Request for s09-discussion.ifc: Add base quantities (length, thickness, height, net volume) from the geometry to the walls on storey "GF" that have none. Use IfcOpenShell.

First a look at what the model holds.

```python
import ifcopenshell
import ifcopenshell.util.element
import ifcopenshell.util.unit

model = ifcopenshell.open("s09-discussion.ifc")
print(model.schema)
for unit_type in ("LENGTHUNIT", "AREAUNIT", "VOLUMEUNIT"):
    print(unit_type, ifcopenshell.util.unit.calculate_unit_scale(model, unit_type))
storey = next(s for s in model.by_type("IfcBuildingStorey") if s.Name == "GF")
walls = [e for e in ifcopenshell.util.element.get_decomposition(storey) if e.is_a("IfcWall")]
for e in sorted(walls, key=lambda e: e.id()):
    print(e.id(), e.is_a(), e.Name, list(ifcopenshell.util.element.get_psets(e, qtos_only=True)), sep=" | ")
```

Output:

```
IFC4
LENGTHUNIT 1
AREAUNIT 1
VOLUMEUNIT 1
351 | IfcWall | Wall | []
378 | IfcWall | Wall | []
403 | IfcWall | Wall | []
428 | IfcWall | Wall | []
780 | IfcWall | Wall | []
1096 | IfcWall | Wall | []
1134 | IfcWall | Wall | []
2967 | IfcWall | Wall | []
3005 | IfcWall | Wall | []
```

```python
import ifcopenshell
import ifcopenshell.api.pset
import ifcopenshell.geom
import ifcopenshell.util.element
import ifcopenshell.util.shape
import ifcopenshell.util.unit

model = ifcopenshell.open("s09-discussion.ifc")
unit_scale = ifcopenshell.util.unit.calculate_unit_scale(model)
volume_scale = ifcopenshell.util.unit.calculate_unit_scale(model, "VOLUMEUNIT")
settings = ifcopenshell.geom.settings()

storey = next(s for s in model.by_type("IfcBuildingStorey") if s.Name == "GF")
walls = [e for e in ifcopenshell.util.element.get_decomposition(storey) if e.is_a("IfcWall")]

for e in sorted(walls, key=lambda e: e.id()):
    if ifcopenshell.util.element.get_psets(e, qtos_only=True, should_inherit=False):
        continue
    # Geometry comes back in metres, in the element's own axes.
    shape = ifcopenshell.geom.create_shape(settings, e)
    values = {
        "Length": ifcopenshell.util.shape.get_x(shape.geometry) / unit_scale,
        "Width": ifcopenshell.util.shape.get_y(shape.geometry) / unit_scale,
        "Height": ifcopenshell.util.shape.get_z(shape.geometry) / unit_scale,
        "NetVolume": ifcopenshell.util.shape.get_volume(shape.geometry) / volume_scale,
    }
    qto = ifcopenshell.api.pset.add_qto(model, product=e, name="Qto_WallBaseQuantities")
    ifcopenshell.api.pset.edit_qto(model, qto=qto, properties=values)
    print(e.id(), {k: round(v, 3) for k, v in values.items()})

model.write("s09-discussion-out.ifc")
```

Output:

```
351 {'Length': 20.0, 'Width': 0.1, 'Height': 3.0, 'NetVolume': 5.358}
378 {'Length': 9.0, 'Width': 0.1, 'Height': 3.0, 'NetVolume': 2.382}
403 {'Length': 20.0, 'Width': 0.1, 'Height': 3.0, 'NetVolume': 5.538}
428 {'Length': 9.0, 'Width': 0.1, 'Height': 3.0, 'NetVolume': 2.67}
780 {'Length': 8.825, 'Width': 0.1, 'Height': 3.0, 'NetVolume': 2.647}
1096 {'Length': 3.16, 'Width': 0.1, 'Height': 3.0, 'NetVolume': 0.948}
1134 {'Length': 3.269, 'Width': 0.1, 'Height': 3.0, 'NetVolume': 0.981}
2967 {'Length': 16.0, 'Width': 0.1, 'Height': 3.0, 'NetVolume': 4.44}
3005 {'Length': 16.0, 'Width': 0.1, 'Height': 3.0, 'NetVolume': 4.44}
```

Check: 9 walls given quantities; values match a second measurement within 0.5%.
